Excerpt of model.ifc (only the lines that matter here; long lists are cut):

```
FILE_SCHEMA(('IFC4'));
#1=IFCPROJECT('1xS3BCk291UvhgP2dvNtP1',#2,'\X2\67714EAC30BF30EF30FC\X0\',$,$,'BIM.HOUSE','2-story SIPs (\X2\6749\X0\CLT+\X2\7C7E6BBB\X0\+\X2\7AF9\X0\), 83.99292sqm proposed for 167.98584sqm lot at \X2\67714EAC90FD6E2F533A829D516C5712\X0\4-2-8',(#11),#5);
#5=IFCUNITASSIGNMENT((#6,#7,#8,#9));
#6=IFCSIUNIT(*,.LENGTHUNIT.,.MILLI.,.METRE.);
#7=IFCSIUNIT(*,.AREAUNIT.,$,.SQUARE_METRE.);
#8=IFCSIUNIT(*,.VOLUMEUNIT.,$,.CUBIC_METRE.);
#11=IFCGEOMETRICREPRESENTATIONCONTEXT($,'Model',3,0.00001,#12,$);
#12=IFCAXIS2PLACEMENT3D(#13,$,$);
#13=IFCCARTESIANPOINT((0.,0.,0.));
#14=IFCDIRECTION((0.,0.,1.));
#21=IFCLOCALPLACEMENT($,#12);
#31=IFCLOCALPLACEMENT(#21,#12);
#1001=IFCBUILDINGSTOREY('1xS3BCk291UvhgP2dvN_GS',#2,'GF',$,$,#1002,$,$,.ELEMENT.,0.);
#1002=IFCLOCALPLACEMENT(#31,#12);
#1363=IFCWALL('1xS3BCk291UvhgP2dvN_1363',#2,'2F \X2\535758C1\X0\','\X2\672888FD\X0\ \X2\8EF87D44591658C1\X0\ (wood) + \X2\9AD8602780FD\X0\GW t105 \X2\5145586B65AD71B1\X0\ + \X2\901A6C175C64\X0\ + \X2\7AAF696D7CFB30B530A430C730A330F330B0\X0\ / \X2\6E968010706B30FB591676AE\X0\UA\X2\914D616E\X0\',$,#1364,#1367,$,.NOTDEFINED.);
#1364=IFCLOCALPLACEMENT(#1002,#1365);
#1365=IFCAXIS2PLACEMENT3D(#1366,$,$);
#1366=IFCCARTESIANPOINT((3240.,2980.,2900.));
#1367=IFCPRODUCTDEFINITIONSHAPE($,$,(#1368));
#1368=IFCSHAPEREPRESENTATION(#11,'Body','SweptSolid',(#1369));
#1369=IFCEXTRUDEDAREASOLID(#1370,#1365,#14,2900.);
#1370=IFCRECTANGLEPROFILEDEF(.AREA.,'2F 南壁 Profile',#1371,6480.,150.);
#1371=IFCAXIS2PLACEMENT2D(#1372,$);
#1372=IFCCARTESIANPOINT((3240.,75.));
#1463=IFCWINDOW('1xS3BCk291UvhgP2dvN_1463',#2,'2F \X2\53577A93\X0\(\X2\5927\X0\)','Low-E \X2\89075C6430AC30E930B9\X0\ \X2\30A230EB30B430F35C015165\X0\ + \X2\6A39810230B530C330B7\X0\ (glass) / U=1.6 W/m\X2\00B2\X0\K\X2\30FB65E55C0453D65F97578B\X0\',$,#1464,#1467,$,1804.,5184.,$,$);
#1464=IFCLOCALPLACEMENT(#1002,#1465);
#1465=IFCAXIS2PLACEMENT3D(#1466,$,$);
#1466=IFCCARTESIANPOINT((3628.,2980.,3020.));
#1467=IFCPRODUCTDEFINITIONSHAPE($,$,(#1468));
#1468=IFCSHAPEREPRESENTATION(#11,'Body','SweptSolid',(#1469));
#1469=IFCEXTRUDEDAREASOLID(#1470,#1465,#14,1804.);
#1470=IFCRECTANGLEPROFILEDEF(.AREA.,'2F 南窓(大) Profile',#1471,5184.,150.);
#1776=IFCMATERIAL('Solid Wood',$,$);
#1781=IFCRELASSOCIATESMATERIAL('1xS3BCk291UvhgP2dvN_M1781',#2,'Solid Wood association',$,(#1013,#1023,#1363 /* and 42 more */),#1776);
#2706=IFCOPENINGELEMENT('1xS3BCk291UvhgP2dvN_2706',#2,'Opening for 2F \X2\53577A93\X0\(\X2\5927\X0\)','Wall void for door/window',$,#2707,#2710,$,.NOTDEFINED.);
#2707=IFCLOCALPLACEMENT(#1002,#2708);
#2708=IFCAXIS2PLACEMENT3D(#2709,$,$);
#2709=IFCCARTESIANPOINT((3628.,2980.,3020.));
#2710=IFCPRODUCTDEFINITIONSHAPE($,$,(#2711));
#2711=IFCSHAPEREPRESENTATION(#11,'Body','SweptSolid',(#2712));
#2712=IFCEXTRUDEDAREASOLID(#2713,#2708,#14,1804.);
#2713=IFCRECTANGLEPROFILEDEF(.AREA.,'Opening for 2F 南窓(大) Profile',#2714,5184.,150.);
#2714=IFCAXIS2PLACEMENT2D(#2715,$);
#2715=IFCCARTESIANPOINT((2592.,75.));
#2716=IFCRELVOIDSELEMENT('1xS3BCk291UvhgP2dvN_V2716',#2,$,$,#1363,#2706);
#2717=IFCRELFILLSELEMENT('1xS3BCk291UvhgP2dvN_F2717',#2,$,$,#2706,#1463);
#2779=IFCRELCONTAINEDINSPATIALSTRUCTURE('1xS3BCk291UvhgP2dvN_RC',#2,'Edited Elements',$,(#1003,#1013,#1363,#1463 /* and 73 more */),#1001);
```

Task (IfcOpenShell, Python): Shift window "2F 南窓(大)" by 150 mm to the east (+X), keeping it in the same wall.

```python
import ifcopenshell
import ifcopenshell.api.geometry
import ifcopenshell.util.placement

model = ifcopenshell.open("model.ifc")

window = model.by_guid("1xS3BCk291UvhgP2dvN_1463")
opening = window.FillsVoids[0].RelatingOpeningElement
wall = opening.VoidsElements[0].RelatingBuildingElement

wall_matrix = ifcopenshell.util.placement.get_local_placement(wall.ObjectPlacement)
shift = wall_matrix[:3, 0] * 150.0
before = ifcopenshell.util.placement.get_local_placement(window.ObjectPlacement)[:3, 3].copy()

# The window is not placed relative to its opening, so move both.
for product in (opening, window):
    matrix = ifcopenshell.util.placement.get_local_placement(product.ObjectPlacement)
    matrix[:3, 3] += shift
    ifcopenshell.api.geometry.edit_object_placement(model, product=product, matrix=matrix, is_si=False)

after = ifcopenshell.util.placement.get_local_placement(window.ObjectPlacement)[:3, 3]
print("window moved by", (after - before).round(3) + 0.0)

model.write("model_rev.ifc")
```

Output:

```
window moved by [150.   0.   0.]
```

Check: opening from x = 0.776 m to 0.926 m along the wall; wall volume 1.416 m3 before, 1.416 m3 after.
